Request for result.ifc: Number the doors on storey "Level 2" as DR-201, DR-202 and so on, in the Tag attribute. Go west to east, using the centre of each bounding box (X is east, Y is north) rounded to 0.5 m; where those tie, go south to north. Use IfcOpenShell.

First a look at what the model holds.

```python
import ifcopenshell
import ifcopenshell.util.element
import ifcopenshell.util.placement

model = ifcopenshell.open("result.ifc")
print(model.schema)
storey = next(s for s in model.by_type("IfcBuildingStorey") if s.Name == "Level 2")
doors = [e for e in ifcopenshell.util.element.get_decomposition(storey) if e.is_a("IfcDoor")]
for e in sorted(doors, key=lambda e: e.id()):
    origin = ifcopenshell.util.placement.get_local_placement(e.ObjectPlacement)[:3, 3]
    print(e.id(), e.Tag, e.Name, origin.round(2) + 0.0, sep=" | ")
```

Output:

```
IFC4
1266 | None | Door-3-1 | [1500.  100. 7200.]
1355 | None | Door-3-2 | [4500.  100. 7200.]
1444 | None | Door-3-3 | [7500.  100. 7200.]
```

```python
import ifcopenshell
import ifcopenshell.geom
import ifcopenshell.util.element
import ifcopenshell.util.shape

model = ifcopenshell.open("result.ifc")
settings = ifcopenshell.geom.settings()
settings.set("use-world-coords", True)


def centre(element):
    shape = ifcopenshell.geom.create_shape(settings, element)
    return ifcopenshell.util.shape.get_bbox_centroid(shape.geometry)


storey = next(s for s in model.by_type("IfcBuildingStorey") if s.Name == "Level 2")
doors = [e for e in ifcopenshell.util.element.get_decomposition(storey) if e.is_a("IfcDoor")]

# Insertion points can sit at a corner or the storey origin, so sort by the geometry (in metres).
centres = {e: centre(e) for e in doors}
doors.sort(key=lambda e: (round(centres[e][0] / 0.5), centres[e][1]))

for i, e in enumerate(doors, start=1):
    number = f"DR-2{i:02d}"
    e.Tag = number
    print(e.id(), number)

model.write("result-out.ifc")
```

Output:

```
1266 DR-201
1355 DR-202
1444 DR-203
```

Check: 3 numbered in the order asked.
